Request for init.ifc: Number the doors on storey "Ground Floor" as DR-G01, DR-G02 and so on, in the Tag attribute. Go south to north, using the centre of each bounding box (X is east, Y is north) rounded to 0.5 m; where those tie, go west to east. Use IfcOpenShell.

First a look at what the model holds.

```python
import ifcopenshell
import ifcopenshell.util.element
import ifcopenshell.util.placement

model = ifcopenshell.open("init.ifc")
print(model.schema)
storey = next(s for s in model.by_type("IfcBuildingStorey") if s.Name == "Ground Floor")
doors = [e for e in ifcopenshell.util.element.get_decomposition(storey) if e.is_a("IfcDoor")]
for e in sorted(doors, key=lambda e: e.id()):
    origin = ifcopenshell.util.placement.get_local_placement(e.ObjectPlacement)[:3, 3]
    print(e.id(), e.Tag, e.Name, origin.round(2) + 0.0, sep=" | ")
```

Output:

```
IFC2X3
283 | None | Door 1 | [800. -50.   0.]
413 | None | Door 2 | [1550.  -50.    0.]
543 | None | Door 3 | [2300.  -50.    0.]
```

```python
import ifcopenshell
import ifcopenshell.geom
import ifcopenshell.util.element
import ifcopenshell.util.shape

model = ifcopenshell.open("init.ifc")
settings = ifcopenshell.geom.settings()
settings.set("use-world-coords", True)


def centre(element):
    shape = ifcopenshell.geom.create_shape(settings, element)
    return ifcopenshell.util.shape.get_bbox_centroid(shape.geometry)


storey = next(s for s in model.by_type("IfcBuildingStorey") if s.Name == "Ground Floor")
doors = [e for e in ifcopenshell.util.element.get_decomposition(storey) if e.is_a("IfcDoor")]

# Insertion points can sit at a corner or the storey origin, so sort by the geometry (in metres).
centres = {e: centre(e) for e in doors}
doors.sort(key=lambda e: (round(centres[e][1] / 0.5), centres[e][0]))

for i, e in enumerate(doors, start=1):
    number = f"DR-G{i:02d}"
    e.Tag = number
    print(e.id(), number)

model.write("init_edited.ifc")
```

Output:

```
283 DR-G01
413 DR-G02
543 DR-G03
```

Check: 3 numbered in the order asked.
